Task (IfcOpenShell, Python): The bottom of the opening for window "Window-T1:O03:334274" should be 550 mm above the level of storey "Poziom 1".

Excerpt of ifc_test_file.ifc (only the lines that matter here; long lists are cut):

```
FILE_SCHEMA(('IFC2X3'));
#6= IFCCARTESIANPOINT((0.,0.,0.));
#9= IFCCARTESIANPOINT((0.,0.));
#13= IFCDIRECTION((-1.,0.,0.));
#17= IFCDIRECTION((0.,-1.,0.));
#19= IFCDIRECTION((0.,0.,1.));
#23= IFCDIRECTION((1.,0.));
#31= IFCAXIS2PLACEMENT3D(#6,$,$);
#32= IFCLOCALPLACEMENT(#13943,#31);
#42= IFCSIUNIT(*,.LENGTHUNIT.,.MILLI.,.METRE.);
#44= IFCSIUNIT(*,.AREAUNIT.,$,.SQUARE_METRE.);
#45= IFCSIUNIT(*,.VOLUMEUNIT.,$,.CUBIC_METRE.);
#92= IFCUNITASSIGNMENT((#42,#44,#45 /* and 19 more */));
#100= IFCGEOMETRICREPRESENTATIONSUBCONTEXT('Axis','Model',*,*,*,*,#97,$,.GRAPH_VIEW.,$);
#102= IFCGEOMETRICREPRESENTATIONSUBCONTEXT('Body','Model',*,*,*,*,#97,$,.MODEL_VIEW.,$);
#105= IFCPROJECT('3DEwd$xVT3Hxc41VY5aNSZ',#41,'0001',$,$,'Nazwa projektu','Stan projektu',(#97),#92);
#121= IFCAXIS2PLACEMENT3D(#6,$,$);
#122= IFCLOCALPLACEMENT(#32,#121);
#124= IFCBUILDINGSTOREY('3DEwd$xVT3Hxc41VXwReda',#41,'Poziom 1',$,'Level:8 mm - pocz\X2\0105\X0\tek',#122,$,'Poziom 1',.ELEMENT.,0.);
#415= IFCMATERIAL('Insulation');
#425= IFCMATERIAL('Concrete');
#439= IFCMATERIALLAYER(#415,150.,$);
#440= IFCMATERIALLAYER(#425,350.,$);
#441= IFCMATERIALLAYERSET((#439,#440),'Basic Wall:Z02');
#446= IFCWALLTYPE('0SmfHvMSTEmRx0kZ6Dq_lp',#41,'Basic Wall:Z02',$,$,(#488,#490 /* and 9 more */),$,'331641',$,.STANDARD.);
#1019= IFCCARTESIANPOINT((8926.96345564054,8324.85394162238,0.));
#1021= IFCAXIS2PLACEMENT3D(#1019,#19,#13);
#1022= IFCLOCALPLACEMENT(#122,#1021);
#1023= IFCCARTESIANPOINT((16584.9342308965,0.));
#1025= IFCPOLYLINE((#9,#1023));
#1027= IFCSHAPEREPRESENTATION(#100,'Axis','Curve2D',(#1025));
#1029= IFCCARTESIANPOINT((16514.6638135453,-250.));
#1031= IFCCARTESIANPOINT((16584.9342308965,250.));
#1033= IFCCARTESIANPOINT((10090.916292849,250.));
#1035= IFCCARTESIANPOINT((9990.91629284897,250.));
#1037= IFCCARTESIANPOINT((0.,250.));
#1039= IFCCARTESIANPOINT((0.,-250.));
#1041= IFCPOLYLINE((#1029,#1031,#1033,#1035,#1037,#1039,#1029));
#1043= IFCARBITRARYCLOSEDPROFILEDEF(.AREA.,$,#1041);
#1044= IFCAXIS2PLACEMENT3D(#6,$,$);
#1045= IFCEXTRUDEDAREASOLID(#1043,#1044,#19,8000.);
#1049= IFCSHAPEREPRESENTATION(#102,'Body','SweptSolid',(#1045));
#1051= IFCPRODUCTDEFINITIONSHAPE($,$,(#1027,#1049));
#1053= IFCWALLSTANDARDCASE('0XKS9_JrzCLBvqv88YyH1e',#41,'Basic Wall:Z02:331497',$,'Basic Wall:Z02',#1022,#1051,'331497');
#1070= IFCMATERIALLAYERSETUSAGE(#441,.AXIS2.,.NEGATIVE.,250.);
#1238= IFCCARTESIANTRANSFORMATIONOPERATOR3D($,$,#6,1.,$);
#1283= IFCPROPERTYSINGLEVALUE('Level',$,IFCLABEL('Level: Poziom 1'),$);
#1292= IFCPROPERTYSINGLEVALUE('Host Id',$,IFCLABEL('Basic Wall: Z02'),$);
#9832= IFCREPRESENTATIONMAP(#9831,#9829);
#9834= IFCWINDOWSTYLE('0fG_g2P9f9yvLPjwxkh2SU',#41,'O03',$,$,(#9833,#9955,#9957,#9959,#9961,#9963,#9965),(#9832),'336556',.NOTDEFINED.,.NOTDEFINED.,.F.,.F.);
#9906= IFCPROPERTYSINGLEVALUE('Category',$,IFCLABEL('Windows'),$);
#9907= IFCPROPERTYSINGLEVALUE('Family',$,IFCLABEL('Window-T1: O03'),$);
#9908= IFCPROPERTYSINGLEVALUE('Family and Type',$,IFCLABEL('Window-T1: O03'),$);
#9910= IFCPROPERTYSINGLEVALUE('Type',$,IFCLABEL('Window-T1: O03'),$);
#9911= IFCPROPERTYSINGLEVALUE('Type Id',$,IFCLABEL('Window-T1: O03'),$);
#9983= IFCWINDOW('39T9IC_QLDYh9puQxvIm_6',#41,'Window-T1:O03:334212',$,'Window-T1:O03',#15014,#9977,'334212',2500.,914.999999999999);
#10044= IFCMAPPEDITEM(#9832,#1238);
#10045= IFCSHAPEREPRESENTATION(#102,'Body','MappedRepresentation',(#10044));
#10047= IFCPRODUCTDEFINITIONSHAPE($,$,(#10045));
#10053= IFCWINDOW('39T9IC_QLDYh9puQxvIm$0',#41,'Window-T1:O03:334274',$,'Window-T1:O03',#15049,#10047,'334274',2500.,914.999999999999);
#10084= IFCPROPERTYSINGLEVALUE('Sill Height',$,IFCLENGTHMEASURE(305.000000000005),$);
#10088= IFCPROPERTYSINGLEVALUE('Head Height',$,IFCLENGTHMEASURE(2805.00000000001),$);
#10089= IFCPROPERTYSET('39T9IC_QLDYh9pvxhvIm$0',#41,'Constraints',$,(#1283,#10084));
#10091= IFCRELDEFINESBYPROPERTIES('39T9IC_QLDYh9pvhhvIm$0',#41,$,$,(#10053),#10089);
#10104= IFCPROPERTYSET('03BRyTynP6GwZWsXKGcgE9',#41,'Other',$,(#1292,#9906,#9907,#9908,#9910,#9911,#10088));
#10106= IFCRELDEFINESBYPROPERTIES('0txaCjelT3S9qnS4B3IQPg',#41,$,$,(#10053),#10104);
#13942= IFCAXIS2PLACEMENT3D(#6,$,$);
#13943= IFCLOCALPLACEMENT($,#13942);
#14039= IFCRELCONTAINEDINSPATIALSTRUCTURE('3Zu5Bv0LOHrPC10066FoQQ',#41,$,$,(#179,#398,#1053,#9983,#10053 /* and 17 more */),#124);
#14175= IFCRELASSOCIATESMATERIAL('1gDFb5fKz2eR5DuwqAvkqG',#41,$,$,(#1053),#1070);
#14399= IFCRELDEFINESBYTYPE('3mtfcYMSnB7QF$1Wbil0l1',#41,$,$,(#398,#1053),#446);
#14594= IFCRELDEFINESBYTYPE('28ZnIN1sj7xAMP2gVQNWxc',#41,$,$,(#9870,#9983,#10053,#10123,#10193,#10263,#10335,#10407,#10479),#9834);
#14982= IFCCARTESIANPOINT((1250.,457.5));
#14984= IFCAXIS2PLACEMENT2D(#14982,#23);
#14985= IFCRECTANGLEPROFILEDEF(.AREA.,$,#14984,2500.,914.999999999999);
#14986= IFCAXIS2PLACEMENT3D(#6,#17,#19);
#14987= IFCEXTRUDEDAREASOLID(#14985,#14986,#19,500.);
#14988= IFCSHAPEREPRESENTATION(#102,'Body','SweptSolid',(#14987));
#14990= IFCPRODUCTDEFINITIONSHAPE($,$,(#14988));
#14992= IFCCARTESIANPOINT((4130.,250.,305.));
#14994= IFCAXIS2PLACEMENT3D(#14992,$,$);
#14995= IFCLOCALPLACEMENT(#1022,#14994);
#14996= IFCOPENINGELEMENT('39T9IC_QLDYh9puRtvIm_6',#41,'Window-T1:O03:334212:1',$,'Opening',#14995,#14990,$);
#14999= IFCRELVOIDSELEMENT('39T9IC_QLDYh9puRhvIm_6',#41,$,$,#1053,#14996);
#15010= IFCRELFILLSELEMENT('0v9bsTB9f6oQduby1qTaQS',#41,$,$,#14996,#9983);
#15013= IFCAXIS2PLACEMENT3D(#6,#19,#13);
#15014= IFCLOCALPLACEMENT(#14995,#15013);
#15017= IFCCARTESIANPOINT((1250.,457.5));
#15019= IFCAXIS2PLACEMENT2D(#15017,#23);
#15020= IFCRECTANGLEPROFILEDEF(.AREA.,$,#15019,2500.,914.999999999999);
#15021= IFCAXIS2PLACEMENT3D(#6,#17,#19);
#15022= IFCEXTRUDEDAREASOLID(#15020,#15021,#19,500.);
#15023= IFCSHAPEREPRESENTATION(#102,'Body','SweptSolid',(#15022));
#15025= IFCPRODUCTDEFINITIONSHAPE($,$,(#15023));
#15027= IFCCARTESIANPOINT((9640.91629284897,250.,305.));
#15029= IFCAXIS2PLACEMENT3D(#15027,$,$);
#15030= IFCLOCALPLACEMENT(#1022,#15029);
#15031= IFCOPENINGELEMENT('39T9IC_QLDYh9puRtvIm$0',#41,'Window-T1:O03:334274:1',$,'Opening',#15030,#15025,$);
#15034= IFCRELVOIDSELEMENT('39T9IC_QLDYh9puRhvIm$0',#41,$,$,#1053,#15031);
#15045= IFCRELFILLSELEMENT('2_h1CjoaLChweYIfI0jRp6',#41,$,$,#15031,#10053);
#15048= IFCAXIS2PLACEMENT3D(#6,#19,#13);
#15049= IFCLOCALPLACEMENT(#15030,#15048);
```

```python
import numpy as np
import ifcopenshell
import ifcopenshell.api.geometry
import ifcopenshell.api.pset
import ifcopenshell.geom
import ifcopenshell.util.element
import ifcopenshell.util.placement
import ifcopenshell.util.shape
import ifcopenshell.util.unit

model = ifcopenshell.open("ifc_test_file.ifc")
unit_scale = ifcopenshell.util.unit.calculate_unit_scale(model)

window = model.by_guid("39T9IC_QLDYh9puQxvIm$0")
opening = window.FillsVoids[0].RelatingOpeningElement
storey = ifcopenshell.util.element.get_container(window, ifc_class="IfcBuildingStorey")
level = ifcopenshell.util.placement.get_local_placement(storey.ObjectPlacement)[2, 3]

# The opening's origin need not be at the sill, so measure its lowest point.
shape = ifcopenshell.geom.create_shape(ifcopenshell.geom.settings(), opening)
bottom = ifcopenshell.util.shape.get_shape_bottom_elevation(shape, shape.geometry) / unit_scale
dz = level + 550.0 - bottom

shift = np.array([0.0, 0.0, dz])
# The window is placed relative to its opening, so it follows when the opening moves.
matrix = ifcopenshell.util.placement.get_local_placement(opening.ObjectPlacement)
matrix[:3, 3] += shift
ifcopenshell.api.geometry.edit_object_placement(
    model, product=opening, matrix=matrix, is_si=False, should_transform_children=True
)

# Keep the stored heights in step.
pset = model.by_id(ifcopenshell.util.element.get_pset(window, "Constraints", should_inherit=False)["id"])
ifcopenshell.api.pset.edit_pset(model, pset=pset, properties={
    "Sill Height": model.create_entity("IfcLengthMeasure", ifcopenshell.util.element.get_pset(window, "Constraints", "Sill Height") + dz),
})
pset = model.by_id(ifcopenshell.util.element.get_pset(window, "Other", should_inherit=False)["id"])
ifcopenshell.api.pset.edit_pset(model, pset=pset, properties={
    "Head Height": model.create_entity("IfcLengthMeasure", ifcopenshell.util.element.get_pset(window, "Other", "Head Height") + dz),
})

print(f"moved by {dz * unit_scale:+.3f} m")

model.write("ifc_test_file-out.ifc")
```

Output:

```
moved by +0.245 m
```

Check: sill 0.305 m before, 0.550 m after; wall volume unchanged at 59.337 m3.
